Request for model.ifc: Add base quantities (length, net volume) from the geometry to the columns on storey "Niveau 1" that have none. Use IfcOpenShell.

First a look at what the model holds.

```python
import ifcopenshell
import ifcopenshell.util.element
import ifcopenshell.util.unit

model = ifcopenshell.open("model.ifc")
print(model.schema)
for unit_type in ("LENGTHUNIT", "AREAUNIT", "VOLUMEUNIT"):
    print(unit_type, ifcopenshell.util.unit.calculate_unit_scale(model, unit_type))
storey = next(s for s in model.by_type("IfcBuildingStorey") if s.Name == "Niveau 1")
columns = [e for e in ifcopenshell.util.element.get_decomposition(storey) if e.is_a("IfcColumn")]
for e in sorted(columns, key=lambda e: e.id()):
    print(e.id(), e.is_a(), e.Name, list(ifcopenshell.util.element.get_psets(e, qtos_only=True)), sep=" | ")
```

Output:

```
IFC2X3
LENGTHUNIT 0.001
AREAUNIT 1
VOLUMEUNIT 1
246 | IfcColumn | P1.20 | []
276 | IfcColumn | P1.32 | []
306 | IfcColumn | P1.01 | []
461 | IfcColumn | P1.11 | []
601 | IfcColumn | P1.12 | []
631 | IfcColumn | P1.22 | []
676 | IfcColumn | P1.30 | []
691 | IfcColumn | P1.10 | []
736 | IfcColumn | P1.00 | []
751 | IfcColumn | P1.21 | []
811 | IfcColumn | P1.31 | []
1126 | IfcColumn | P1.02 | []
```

```python
import ifcopenshell
import ifcopenshell.api.pset
import ifcopenshell.geom
import ifcopenshell.util.element
import ifcopenshell.util.shape
import ifcopenshell.util.unit

model = ifcopenshell.open("model.ifc")
unit_scale = ifcopenshell.util.unit.calculate_unit_scale(model)
volume_scale = ifcopenshell.util.unit.calculate_unit_scale(model, "VOLUMEUNIT")
settings = ifcopenshell.geom.settings()

storey = next(s for s in model.by_type("IfcBuildingStorey") if s.Name == "Niveau 1")
columns = [e for e in ifcopenshell.util.element.get_decomposition(storey) if e.is_a("IfcColumn")]

for e in sorted(columns, key=lambda e: e.id()):
    if ifcopenshell.util.element.get_psets(e, qtos_only=True, should_inherit=False):
        continue
    # Geometry comes back in metres, in the element's own axes.
    shape = ifcopenshell.geom.create_shape(settings, e)
    values = {
        "Length": ifcopenshell.util.shape.get_z(shape.geometry) / unit_scale,
        "NetVolume": ifcopenshell.util.shape.get_volume(shape.geometry) / volume_scale,
    }
    qto = ifcopenshell.api.pset.add_qto(model, product=e, name="BaseQuantities")
    ifcopenshell.api.pset.edit_qto(model, qto=qto, properties=values)
    print(e.id(), {k: round(v, 3) for k, v in values.items()})

model.write("model-out.ifc")
```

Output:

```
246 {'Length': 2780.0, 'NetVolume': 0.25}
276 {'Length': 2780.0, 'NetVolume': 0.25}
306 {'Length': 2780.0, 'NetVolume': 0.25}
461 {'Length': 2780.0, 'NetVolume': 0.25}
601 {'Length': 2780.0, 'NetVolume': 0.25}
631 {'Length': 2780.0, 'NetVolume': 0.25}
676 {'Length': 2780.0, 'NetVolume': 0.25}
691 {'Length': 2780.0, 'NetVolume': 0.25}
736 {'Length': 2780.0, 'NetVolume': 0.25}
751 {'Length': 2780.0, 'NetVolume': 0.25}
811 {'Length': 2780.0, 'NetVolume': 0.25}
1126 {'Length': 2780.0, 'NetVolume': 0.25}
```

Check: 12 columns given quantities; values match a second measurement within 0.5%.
